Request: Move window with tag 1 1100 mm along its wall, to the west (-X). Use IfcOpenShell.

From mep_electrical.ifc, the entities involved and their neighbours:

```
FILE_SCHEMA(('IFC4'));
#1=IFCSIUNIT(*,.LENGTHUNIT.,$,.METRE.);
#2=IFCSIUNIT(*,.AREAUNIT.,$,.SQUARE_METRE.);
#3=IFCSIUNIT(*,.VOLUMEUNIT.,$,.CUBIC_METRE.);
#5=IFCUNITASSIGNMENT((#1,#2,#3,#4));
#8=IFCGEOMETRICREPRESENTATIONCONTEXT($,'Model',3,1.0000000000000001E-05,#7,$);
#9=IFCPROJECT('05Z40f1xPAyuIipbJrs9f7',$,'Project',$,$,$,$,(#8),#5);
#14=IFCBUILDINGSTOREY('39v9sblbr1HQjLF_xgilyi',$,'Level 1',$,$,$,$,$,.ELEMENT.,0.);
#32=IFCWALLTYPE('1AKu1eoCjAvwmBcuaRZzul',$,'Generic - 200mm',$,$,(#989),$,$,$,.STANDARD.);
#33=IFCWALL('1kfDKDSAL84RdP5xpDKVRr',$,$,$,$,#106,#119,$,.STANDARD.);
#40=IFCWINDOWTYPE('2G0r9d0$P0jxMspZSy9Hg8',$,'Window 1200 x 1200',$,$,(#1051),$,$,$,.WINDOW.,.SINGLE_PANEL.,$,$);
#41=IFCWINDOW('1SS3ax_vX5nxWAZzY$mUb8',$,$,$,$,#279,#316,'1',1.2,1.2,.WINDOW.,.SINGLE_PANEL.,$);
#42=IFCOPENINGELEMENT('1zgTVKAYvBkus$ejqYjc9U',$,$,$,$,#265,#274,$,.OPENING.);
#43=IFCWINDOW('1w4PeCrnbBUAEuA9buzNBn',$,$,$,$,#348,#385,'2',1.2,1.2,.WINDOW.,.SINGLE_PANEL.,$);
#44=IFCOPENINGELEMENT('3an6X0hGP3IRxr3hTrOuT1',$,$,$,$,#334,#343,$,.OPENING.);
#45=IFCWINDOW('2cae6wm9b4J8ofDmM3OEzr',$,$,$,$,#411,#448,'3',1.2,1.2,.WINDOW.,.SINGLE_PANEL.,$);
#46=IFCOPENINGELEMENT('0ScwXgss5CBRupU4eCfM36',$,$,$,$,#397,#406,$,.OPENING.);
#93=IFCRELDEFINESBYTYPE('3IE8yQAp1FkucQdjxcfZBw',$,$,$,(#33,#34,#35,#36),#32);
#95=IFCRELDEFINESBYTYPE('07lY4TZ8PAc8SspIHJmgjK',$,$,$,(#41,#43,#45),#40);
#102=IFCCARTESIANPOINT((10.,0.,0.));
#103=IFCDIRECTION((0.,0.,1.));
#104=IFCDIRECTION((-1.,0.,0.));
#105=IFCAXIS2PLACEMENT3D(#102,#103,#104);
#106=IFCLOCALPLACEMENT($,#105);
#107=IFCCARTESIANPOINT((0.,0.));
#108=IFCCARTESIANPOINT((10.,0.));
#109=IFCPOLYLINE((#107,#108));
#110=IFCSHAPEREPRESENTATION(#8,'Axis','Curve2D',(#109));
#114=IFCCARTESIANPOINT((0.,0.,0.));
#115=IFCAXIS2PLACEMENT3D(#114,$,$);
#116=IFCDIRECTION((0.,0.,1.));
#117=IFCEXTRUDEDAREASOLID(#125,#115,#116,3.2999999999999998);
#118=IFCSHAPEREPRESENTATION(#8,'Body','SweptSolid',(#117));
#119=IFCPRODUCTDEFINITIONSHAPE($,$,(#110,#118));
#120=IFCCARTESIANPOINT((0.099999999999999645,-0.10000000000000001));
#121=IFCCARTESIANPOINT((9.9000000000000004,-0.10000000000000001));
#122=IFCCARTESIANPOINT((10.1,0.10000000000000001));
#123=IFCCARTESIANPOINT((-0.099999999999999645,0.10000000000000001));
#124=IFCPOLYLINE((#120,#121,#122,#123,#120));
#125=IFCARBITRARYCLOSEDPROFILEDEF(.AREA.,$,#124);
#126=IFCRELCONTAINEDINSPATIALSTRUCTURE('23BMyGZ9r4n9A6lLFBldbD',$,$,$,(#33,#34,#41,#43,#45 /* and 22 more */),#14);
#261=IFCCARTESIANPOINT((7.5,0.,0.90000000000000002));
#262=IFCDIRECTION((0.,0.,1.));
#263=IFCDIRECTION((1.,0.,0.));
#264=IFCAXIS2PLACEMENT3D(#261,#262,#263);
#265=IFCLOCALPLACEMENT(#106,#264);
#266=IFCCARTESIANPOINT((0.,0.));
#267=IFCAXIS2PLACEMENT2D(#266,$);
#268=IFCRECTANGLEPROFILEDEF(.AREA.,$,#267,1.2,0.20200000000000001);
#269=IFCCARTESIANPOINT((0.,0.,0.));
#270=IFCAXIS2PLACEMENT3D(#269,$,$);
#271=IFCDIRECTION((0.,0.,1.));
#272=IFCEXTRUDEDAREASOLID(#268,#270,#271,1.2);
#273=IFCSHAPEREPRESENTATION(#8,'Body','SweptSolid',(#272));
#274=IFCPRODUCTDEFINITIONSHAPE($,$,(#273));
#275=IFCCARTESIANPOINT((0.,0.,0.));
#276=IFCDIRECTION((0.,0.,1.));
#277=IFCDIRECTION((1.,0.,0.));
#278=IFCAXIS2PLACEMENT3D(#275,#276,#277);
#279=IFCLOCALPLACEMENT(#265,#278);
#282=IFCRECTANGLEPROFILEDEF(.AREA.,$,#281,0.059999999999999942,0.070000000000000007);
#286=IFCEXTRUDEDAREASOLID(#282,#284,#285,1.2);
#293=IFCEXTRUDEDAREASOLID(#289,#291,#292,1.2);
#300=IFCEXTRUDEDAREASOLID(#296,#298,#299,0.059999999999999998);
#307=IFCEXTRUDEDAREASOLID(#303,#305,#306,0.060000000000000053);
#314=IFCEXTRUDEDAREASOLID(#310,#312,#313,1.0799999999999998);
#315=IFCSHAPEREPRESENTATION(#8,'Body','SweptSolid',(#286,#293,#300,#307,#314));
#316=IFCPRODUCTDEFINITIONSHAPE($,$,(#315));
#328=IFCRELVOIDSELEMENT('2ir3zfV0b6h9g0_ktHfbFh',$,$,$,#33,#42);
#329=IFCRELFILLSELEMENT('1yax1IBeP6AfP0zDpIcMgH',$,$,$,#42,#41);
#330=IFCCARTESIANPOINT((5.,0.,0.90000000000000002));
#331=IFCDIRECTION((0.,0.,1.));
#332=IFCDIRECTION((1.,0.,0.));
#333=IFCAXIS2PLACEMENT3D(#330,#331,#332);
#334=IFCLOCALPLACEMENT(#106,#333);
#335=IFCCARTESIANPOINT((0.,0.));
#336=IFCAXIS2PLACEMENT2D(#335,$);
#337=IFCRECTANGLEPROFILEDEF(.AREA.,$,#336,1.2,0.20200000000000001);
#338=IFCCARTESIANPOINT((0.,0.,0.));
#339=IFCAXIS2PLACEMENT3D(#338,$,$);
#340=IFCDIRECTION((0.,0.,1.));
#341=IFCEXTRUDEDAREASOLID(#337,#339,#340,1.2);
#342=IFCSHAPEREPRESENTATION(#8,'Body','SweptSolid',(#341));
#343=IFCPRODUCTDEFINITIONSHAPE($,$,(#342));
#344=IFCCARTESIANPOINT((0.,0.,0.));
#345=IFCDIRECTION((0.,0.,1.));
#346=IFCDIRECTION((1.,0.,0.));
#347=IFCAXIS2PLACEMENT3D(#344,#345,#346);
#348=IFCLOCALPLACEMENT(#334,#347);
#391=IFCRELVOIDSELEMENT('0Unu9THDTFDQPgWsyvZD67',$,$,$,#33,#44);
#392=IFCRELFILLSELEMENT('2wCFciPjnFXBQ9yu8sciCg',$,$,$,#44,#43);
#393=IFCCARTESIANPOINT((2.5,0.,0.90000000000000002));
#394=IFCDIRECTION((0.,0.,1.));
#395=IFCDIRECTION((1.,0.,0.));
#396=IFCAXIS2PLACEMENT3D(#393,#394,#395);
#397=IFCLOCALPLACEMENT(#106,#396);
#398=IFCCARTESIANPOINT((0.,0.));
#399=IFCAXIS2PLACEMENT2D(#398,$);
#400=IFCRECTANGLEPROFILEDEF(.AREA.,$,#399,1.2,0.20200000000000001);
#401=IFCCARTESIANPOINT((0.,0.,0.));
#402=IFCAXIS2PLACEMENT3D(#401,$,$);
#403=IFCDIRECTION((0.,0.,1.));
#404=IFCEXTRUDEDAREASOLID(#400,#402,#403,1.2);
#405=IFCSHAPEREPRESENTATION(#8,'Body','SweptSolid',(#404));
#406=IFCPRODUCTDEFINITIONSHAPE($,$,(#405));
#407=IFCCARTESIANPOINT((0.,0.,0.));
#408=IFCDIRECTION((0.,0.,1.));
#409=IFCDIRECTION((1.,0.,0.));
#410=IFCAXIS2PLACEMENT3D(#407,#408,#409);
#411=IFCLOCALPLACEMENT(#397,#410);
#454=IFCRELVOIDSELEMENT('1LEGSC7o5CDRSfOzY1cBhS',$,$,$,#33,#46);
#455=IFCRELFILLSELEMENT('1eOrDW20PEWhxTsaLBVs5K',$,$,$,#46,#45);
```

```python
import ifcopenshell
import ifcopenshell.api.geometry
import ifcopenshell.util.placement
import ifcopenshell.util.unit

model = ifcopenshell.open("mep_electrical.ifc")
unit_scale = ifcopenshell.util.unit.calculate_unit_scale(model)

window = model.by_guid("1SS3ax_vX5nxWAZzY$mUb8")
opening = window.FillsVoids[0].RelatingOpeningElement
wall = opening.VoidsElements[0].RelatingBuildingElement

wall_matrix = ifcopenshell.util.placement.get_local_placement(wall.ObjectPlacement)
shift = wall_matrix[:3, 0] * 1.1 / unit_scale
before = ifcopenshell.util.placement.get_local_placement(window.ObjectPlacement)[:3, 3].copy()

# The window is placed relative to its opening, so it follows when the opening moves.
matrix = ifcopenshell.util.placement.get_local_placement(opening.ObjectPlacement)
matrix[:3, 3] += shift
ifcopenshell.api.geometry.edit_object_placement(
    model, product=opening, matrix=matrix, is_si=False, should_transform_children=True
)

after = ifcopenshell.util.placement.get_local_placement(window.ObjectPlacement)[:3, 3]
print("window moved by", (after - before).round(3) + 0.0)

model.write("mep_electrical_edited.ifc")
```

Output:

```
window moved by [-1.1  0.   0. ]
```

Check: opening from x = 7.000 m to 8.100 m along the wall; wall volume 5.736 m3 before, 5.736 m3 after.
